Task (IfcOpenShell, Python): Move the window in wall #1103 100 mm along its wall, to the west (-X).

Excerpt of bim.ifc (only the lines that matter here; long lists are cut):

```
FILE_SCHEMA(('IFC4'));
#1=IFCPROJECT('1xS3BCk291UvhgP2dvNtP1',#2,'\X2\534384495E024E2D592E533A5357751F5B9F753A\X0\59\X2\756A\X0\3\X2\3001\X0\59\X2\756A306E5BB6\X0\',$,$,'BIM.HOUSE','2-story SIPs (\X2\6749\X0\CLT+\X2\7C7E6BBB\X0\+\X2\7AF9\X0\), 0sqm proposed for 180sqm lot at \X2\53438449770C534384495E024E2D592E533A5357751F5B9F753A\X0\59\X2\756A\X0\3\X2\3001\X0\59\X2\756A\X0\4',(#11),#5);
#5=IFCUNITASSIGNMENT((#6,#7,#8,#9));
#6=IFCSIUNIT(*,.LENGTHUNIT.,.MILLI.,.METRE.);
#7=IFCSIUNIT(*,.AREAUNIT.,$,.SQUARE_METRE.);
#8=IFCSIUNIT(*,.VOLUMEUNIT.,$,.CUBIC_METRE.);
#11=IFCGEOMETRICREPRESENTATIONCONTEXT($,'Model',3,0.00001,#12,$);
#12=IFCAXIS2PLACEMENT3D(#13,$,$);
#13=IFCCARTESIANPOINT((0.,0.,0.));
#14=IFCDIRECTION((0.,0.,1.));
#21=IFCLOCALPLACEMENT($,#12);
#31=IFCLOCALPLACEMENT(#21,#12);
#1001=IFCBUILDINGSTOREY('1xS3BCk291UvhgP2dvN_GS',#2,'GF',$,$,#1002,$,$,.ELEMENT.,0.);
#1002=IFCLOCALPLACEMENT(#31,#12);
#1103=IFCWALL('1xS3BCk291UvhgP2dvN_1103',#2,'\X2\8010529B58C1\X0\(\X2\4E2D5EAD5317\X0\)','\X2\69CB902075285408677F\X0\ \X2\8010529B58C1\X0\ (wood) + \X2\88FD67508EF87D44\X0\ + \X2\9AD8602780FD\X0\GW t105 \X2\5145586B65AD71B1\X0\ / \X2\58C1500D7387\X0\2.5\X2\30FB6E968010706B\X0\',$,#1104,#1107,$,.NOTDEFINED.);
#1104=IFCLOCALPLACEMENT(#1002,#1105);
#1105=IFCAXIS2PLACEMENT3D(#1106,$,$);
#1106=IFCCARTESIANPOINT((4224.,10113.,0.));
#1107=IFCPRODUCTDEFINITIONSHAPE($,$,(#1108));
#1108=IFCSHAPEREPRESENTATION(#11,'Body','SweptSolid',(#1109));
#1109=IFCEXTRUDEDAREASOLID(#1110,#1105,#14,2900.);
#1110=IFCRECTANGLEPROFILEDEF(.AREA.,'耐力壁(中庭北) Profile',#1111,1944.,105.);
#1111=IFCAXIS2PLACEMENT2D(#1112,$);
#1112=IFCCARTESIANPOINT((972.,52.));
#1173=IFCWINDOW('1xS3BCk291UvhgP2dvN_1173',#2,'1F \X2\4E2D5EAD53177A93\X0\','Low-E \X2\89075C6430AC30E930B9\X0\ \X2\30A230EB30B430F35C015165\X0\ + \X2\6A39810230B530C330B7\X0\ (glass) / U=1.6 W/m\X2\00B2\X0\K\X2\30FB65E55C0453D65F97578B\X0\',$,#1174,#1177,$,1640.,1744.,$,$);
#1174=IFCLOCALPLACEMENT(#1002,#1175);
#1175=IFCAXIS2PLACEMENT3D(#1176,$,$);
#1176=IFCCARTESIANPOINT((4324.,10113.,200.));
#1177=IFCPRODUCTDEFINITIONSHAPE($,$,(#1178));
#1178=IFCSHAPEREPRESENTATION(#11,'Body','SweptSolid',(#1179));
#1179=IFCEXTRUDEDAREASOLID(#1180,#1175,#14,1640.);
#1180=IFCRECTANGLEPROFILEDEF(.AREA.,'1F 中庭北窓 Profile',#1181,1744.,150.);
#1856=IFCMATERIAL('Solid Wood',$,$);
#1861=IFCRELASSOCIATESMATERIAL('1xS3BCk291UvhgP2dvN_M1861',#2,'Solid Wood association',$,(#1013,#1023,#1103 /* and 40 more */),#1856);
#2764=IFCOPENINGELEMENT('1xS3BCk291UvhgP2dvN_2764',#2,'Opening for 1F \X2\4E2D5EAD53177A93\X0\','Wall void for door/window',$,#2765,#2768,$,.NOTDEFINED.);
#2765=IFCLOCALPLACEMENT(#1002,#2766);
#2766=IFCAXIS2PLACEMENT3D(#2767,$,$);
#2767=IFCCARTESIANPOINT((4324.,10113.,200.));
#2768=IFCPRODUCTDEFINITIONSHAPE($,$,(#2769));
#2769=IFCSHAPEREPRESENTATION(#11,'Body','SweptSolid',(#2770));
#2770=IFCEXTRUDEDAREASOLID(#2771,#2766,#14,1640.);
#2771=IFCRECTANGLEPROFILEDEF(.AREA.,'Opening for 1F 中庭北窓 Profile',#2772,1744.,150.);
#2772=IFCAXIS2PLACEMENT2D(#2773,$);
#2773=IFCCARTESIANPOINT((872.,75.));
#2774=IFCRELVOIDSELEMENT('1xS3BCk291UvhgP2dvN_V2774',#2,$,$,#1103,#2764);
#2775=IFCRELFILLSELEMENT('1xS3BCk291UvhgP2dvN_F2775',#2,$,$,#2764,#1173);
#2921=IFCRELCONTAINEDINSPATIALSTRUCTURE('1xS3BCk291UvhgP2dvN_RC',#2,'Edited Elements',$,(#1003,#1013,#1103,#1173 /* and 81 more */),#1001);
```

```python
import ifcopenshell
import ifcopenshell.api.geometry
import ifcopenshell.util.placement
import ifcopenshell.util.unit

model = ifcopenshell.open("bim.ifc")
unit_scale = ifcopenshell.util.unit.calculate_unit_scale(model)

window = model.by_guid("1xS3BCk291UvhgP2dvN_1173")
opening = window.FillsVoids[0].RelatingOpeningElement
wall = opening.VoidsElements[0].RelatingBuildingElement

wall_matrix = ifcopenshell.util.placement.get_local_placement(wall.ObjectPlacement)
shift = wall_matrix[:3, 0] * -0.1 / unit_scale
before = ifcopenshell.util.placement.get_local_placement(window.ObjectPlacement)[:3, 3].copy()

# The window is not placed relative to its opening, so move both.
for product in (opening, window):
    matrix = ifcopenshell.util.placement.get_local_placement(product.ObjectPlacement)
    matrix[:3, 3] += shift
    ifcopenshell.api.geometry.edit_object_placement(model, product=product, matrix=matrix, is_si=False)

after = ifcopenshell.util.placement.get_local_placement(window.ObjectPlacement)[:3, 3]
print("window moved by", (after - before).round(3) + 0.0)

model.write("bim-out.ifc")
```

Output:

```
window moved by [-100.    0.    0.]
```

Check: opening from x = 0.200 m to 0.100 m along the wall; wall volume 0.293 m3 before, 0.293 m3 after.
